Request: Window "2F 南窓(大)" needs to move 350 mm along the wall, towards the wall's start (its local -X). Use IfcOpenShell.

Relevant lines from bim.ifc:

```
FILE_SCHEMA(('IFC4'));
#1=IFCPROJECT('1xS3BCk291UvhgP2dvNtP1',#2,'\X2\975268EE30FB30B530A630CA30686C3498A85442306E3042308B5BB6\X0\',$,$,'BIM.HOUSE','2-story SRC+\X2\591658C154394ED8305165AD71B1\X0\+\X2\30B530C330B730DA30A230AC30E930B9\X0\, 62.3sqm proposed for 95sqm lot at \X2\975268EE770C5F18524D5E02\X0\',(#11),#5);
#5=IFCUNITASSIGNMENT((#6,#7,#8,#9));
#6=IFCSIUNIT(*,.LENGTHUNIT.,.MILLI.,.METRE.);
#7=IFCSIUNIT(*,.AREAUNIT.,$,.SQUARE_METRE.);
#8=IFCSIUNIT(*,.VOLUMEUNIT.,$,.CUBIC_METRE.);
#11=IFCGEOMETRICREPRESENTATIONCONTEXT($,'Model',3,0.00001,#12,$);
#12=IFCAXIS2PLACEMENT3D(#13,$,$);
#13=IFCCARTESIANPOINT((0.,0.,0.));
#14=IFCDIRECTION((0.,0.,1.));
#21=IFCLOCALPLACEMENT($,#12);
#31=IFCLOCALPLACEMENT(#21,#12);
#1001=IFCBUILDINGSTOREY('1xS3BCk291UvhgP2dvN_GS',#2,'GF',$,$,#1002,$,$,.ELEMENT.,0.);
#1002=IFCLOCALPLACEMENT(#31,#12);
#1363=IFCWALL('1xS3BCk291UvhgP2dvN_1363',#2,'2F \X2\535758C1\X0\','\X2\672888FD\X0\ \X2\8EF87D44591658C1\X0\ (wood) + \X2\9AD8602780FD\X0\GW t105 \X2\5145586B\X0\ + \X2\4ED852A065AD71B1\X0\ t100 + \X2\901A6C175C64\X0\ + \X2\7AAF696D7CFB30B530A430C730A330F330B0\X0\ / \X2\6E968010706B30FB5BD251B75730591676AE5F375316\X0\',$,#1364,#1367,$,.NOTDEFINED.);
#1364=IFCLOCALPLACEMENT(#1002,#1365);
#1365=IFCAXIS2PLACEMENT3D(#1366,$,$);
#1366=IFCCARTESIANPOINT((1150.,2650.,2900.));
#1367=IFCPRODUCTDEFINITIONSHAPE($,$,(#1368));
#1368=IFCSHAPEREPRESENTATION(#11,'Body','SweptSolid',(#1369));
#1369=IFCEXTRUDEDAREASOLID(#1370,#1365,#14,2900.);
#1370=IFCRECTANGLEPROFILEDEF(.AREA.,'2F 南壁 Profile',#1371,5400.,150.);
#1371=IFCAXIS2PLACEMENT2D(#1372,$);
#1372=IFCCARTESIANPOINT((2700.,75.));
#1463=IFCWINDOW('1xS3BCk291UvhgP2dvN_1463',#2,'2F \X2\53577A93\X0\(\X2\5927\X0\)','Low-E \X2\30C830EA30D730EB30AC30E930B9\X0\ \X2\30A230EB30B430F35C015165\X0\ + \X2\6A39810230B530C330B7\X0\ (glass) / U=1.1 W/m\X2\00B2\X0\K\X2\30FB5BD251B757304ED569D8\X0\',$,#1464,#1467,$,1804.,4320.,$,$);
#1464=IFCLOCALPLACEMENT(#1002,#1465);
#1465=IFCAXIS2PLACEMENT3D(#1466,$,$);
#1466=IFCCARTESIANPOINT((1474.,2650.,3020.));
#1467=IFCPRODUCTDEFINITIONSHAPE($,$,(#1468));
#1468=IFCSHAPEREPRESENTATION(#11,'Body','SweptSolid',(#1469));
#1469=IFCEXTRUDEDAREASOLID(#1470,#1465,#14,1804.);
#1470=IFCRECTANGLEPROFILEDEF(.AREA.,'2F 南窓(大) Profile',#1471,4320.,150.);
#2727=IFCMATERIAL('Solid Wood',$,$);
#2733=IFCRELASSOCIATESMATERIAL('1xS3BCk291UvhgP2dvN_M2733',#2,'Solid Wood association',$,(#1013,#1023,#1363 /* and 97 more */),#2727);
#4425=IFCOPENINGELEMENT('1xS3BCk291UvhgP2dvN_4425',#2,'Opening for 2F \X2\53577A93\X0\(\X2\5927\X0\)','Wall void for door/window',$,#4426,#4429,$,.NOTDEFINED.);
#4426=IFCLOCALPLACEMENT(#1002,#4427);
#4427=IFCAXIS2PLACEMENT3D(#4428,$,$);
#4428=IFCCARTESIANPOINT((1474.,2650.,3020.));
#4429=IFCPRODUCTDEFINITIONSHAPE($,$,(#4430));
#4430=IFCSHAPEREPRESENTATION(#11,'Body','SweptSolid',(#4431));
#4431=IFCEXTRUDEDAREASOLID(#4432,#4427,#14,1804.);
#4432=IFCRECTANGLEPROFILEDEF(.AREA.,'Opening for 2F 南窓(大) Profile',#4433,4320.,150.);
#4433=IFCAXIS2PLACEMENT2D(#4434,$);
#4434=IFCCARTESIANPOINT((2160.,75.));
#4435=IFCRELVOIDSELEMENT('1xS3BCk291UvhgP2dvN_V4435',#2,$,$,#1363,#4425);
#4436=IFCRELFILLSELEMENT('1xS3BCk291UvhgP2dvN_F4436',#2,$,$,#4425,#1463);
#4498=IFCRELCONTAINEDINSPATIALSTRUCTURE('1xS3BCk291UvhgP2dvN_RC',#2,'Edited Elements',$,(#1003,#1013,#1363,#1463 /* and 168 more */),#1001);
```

```python
import ifcopenshell
import ifcopenshell.api.geometry
import ifcopenshell.util.placement

model = ifcopenshell.open("bim.ifc")

window = model.by_guid("1xS3BCk291UvhgP2dvN_1463")
opening = window.FillsVoids[0].RelatingOpeningElement
wall = opening.VoidsElements[0].RelatingBuildingElement

wall_matrix = ifcopenshell.util.placement.get_local_placement(wall.ObjectPlacement)
shift = wall_matrix[:3, 0] * -350.0
before = ifcopenshell.util.placement.get_local_placement(window.ObjectPlacement)[:3, 3].copy()

# The window is not placed relative to its opening, so move both.
for product in (opening, window):
    matrix = ifcopenshell.util.placement.get_local_placement(product.ObjectPlacement)
    matrix[:3, 3] += shift
    ifcopenshell.api.geometry.edit_object_placement(model, product=product, matrix=matrix, is_si=False)

after = ifcopenshell.util.placement.get_local_placement(window.ObjectPlacement)[:3, 3]
print("window moved by", (after - before).round(3) + 0.0)

model.write("bim_edited.ifc")
```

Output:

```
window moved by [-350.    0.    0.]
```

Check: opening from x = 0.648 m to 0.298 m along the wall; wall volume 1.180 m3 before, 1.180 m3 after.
